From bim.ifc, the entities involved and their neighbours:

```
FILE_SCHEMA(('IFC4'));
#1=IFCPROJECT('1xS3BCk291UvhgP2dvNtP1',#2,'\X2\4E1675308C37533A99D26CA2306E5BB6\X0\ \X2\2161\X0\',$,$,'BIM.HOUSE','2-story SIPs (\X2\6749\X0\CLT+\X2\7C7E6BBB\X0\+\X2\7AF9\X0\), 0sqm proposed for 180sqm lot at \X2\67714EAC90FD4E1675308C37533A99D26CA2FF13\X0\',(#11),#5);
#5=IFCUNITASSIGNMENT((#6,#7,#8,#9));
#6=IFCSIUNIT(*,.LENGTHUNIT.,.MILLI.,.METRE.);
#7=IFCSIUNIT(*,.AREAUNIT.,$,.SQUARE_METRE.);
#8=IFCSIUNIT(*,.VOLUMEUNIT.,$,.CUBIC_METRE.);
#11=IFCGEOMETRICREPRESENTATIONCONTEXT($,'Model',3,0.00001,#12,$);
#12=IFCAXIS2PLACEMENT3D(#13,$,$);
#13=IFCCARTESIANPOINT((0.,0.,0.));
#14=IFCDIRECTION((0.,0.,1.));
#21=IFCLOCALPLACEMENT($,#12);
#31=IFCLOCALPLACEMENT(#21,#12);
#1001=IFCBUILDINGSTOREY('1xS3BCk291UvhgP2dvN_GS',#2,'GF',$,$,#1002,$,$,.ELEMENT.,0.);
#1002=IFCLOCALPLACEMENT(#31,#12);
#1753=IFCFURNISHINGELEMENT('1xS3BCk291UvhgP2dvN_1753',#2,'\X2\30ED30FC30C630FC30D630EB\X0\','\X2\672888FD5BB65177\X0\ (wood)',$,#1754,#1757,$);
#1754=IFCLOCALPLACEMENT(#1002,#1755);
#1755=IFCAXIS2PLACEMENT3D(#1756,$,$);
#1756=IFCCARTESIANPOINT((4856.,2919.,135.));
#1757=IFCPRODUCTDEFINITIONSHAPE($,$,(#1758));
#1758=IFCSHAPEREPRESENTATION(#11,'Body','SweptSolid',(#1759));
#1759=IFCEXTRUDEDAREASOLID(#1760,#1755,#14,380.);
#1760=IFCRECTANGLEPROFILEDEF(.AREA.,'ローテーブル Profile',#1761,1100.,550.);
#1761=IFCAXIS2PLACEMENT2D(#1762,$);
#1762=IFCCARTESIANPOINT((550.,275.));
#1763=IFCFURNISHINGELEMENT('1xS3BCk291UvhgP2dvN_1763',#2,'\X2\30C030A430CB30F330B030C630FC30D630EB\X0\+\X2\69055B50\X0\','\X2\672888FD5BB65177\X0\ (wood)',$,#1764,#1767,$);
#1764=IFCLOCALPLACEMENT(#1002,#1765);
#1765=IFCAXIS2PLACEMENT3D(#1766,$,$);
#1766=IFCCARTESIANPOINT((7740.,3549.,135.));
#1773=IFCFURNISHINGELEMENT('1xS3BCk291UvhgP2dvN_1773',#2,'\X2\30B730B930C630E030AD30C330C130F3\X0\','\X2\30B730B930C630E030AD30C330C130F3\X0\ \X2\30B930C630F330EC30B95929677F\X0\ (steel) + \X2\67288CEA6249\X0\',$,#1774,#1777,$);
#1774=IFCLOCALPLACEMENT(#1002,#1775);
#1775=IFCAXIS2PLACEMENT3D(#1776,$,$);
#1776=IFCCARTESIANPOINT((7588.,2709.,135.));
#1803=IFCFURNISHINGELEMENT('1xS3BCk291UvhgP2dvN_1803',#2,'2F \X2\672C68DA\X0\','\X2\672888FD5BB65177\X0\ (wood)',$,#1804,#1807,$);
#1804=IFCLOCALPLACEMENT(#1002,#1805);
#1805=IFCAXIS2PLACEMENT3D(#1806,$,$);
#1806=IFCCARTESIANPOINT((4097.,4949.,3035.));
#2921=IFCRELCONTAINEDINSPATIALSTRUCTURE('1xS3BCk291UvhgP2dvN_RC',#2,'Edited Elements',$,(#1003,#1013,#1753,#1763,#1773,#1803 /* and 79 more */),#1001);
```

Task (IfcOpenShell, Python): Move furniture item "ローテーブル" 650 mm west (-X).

```python
import ifcopenshell
import ifcopenshell.api.geometry
import ifcopenshell.util.placement
import ifcopenshell.util.unit

model = ifcopenshell.open("bim.ifc")
unit_scale = ifcopenshell.util.unit.calculate_unit_scale(model)

item = model.by_guid("1xS3BCk291UvhgP2dvN_1753")
matrix = ifcopenshell.util.placement.get_local_placement(item.ObjectPlacement)
matrix[0, 3] -= 0.65 / unit_scale
ifcopenshell.api.geometry.edit_object_placement(model, product=item, matrix=matrix, is_si=False)

print(ifcopenshell.util.placement.get_local_placement(item.ObjectPlacement).round(3) + 0.0)

model.write("bim_edited.ifc")
```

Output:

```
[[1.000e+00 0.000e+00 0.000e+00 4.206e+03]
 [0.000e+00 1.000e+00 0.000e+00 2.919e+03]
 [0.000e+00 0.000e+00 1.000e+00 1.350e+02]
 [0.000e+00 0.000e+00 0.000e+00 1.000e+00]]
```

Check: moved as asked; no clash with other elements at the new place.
